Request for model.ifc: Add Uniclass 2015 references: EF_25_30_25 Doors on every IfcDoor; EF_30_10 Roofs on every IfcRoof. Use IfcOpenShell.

First a look at what the model holds.

```python
import ifcopenshell

model = ifcopenshell.open("model.ifc")
print(model.schema)
print("classifications:", [c.Name for c in model.by_type("IfcClassification")])
for ifc_class in ("IfcDoor", "IfcRoof", "IfcStair", "IfcWall", "IfcWindow"):
    print(ifc_class, len(model.by_type(ifc_class)))
```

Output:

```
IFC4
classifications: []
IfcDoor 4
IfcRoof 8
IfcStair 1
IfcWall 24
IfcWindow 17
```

```python
import ifcopenshell
import ifcopenshell.api.classification

model = ifcopenshell.open("model.ifc")

system = ifcopenshell.api.classification.add_classification(model, classification="Uniclass 2015")

codes = {
    "IfcDoor": ("EF_25_30_25", "Doors"),
    "IfcRoof": ("EF_30_10", "Roofs"),
}
for ifc_class, (code, name) in codes.items():
    products = model.by_type(ifc_class)
    ifcopenshell.api.classification.add_reference(
        model, products=products, classification=system, identification=code, name=name
    )
    print(code, len(products))

model.write("model-out.ifc")
```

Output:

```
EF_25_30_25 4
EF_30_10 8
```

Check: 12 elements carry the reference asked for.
